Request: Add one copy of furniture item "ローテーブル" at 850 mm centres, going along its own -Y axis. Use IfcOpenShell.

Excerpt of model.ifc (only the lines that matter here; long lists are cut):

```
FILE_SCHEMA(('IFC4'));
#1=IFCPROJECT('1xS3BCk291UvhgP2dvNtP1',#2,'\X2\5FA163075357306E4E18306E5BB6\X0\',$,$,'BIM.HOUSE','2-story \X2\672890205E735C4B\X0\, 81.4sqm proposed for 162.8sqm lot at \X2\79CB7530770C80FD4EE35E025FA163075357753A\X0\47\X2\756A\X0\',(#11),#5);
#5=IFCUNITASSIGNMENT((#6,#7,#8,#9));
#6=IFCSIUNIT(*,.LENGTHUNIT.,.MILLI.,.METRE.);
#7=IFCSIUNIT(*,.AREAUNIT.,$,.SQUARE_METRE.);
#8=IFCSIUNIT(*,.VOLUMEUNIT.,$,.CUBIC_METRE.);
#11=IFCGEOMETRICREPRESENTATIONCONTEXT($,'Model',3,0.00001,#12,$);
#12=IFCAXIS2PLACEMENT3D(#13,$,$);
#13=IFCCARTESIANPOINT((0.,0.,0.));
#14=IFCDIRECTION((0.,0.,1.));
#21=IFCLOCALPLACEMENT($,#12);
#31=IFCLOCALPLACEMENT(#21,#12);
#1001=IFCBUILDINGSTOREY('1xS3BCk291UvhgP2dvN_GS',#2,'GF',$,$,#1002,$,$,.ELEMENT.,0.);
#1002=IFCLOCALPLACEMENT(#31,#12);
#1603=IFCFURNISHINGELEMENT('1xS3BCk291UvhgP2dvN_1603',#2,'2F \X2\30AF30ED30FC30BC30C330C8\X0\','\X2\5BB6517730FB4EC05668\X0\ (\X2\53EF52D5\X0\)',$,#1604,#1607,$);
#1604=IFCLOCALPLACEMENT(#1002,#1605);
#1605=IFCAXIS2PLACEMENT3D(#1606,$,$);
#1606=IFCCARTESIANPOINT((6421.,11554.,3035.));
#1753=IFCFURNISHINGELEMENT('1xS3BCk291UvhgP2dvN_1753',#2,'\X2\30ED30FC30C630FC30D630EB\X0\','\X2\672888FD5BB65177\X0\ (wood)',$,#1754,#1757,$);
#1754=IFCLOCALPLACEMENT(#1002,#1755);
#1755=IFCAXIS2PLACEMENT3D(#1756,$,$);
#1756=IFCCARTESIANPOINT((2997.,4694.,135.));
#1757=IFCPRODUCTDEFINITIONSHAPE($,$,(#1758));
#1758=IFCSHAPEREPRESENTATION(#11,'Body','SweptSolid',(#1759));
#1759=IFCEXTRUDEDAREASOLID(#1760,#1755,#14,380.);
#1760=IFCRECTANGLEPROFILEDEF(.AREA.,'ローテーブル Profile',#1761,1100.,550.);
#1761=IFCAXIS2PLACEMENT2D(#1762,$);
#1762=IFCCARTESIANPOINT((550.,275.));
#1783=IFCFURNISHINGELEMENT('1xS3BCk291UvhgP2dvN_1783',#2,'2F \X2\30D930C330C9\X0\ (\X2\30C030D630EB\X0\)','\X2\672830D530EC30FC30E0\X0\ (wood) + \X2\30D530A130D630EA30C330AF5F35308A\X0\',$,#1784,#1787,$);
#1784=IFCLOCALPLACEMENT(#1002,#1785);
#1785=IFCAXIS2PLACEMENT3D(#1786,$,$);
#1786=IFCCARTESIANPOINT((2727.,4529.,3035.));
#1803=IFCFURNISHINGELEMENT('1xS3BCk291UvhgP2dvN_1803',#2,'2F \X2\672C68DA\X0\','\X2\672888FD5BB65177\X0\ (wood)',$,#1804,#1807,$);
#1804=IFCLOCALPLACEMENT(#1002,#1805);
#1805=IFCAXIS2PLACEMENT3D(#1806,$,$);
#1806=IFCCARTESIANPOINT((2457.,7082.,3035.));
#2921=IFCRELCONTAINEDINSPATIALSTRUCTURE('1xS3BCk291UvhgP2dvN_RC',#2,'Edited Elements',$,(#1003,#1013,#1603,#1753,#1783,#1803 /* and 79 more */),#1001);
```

```python
import ifcopenshell
import ifcopenshell.api.geometry
import ifcopenshell.api.root
import ifcopenshell.util.element
import ifcopenshell.util.placement
import ifcopenshell.util.unit

model = ifcopenshell.open("model.ifc")
unit_scale = ifcopenshell.util.unit.calculate_unit_scale(model)


def reuse_history(source, copy):
    """copy_class also copies each property set's owner history, people and application; keep the originals."""
    for rel in copy.IsDefinedBy:
        if rel.is_a("IfcRelDefinesByProperties") and (history := rel.RelatingPropertyDefinition.OwnerHistory):
            rel.RelatingPropertyDefinition.OwnerHistory = source.OwnerHistory
            ifcopenshell.util.element.remove_deep2(model, history)


source = model.by_guid("1xS3BCk291UvhgP2dvN_1753")
base = ifcopenshell.util.placement.get_local_placement(source.ObjectPlacement)
step = -base[:3, 1] * 0.85 / unit_scale

for i in range(1, 2):
    copy = ifcopenshell.api.root.copy_class(model, product=source)
    copy.Representation = ifcopenshell.util.element.copy_deep(
        model, source.Representation, exclude=["IfcGeometricRepresentationContext", "IfcRepresentationMap"]
    )
    reuse_history(source, copy)
    matrix = base.copy()
    matrix[:3, 3] += i * step
    print("added at", matrix[:3, 3].round(3) + 0.0)
    ifcopenshell.api.geometry.edit_object_placement(model, product=copy, matrix=matrix, is_si=False)

model.write("model_edited.ifc")
```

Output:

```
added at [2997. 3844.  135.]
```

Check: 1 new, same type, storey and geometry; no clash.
